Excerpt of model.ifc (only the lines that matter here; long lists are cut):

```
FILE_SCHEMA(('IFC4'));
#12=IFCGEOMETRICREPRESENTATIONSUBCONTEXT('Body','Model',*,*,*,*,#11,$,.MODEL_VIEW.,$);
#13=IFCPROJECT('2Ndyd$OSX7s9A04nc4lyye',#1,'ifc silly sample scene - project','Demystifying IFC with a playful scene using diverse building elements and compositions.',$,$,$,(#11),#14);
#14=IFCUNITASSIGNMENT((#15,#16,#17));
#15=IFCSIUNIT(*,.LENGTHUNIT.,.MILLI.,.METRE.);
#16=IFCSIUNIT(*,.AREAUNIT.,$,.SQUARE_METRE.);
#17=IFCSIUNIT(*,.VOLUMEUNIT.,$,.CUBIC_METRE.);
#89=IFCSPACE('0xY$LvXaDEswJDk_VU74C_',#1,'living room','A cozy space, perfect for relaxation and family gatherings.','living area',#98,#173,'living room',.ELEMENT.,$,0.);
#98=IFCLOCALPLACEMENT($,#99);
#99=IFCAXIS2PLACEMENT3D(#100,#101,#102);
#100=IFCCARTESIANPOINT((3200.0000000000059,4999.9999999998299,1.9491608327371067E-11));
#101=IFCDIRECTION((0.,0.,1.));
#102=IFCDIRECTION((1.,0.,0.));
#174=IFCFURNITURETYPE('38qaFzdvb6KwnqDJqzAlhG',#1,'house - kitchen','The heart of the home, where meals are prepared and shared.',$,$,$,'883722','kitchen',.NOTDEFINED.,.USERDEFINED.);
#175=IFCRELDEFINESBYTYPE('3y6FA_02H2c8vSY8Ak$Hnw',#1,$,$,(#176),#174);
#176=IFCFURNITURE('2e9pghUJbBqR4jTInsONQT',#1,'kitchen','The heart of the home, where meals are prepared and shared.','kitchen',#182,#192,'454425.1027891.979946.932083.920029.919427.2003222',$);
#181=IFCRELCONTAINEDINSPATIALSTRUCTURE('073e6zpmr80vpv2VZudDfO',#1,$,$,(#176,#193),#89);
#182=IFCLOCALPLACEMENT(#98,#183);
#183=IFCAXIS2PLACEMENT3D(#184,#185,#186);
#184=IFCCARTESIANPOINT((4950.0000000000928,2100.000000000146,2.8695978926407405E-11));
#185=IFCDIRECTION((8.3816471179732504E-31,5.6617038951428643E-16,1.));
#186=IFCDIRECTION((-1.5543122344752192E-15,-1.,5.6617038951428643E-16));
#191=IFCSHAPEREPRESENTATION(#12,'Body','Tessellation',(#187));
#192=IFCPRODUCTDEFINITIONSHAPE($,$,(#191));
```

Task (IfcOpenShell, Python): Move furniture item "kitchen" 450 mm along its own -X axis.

```python
import ifcopenshell
import ifcopenshell.api.geometry
import ifcopenshell.util.placement
import ifcopenshell.util.unit

model = ifcopenshell.open("model.ifc")
unit_scale = ifcopenshell.util.unit.calculate_unit_scale(model)

item = model.by_guid("2e9pghUJbBqR4jTInsONQT")
matrix = ifcopenshell.util.placement.get_local_placement(item.ObjectPlacement)
matrix[:3, 3] -= matrix[:3, 0] * 0.45 / unit_scale
ifcopenshell.api.geometry.edit_object_placement(model, product=item, matrix=matrix, is_si=False)

print(ifcopenshell.util.placement.get_local_placement(item.ObjectPlacement).round(3) + 0.0)

model.write("model-out.ifc")
```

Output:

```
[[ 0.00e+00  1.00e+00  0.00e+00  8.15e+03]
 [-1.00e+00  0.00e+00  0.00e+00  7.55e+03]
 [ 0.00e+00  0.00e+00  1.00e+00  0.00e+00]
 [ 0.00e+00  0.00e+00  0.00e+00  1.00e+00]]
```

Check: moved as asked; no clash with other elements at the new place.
